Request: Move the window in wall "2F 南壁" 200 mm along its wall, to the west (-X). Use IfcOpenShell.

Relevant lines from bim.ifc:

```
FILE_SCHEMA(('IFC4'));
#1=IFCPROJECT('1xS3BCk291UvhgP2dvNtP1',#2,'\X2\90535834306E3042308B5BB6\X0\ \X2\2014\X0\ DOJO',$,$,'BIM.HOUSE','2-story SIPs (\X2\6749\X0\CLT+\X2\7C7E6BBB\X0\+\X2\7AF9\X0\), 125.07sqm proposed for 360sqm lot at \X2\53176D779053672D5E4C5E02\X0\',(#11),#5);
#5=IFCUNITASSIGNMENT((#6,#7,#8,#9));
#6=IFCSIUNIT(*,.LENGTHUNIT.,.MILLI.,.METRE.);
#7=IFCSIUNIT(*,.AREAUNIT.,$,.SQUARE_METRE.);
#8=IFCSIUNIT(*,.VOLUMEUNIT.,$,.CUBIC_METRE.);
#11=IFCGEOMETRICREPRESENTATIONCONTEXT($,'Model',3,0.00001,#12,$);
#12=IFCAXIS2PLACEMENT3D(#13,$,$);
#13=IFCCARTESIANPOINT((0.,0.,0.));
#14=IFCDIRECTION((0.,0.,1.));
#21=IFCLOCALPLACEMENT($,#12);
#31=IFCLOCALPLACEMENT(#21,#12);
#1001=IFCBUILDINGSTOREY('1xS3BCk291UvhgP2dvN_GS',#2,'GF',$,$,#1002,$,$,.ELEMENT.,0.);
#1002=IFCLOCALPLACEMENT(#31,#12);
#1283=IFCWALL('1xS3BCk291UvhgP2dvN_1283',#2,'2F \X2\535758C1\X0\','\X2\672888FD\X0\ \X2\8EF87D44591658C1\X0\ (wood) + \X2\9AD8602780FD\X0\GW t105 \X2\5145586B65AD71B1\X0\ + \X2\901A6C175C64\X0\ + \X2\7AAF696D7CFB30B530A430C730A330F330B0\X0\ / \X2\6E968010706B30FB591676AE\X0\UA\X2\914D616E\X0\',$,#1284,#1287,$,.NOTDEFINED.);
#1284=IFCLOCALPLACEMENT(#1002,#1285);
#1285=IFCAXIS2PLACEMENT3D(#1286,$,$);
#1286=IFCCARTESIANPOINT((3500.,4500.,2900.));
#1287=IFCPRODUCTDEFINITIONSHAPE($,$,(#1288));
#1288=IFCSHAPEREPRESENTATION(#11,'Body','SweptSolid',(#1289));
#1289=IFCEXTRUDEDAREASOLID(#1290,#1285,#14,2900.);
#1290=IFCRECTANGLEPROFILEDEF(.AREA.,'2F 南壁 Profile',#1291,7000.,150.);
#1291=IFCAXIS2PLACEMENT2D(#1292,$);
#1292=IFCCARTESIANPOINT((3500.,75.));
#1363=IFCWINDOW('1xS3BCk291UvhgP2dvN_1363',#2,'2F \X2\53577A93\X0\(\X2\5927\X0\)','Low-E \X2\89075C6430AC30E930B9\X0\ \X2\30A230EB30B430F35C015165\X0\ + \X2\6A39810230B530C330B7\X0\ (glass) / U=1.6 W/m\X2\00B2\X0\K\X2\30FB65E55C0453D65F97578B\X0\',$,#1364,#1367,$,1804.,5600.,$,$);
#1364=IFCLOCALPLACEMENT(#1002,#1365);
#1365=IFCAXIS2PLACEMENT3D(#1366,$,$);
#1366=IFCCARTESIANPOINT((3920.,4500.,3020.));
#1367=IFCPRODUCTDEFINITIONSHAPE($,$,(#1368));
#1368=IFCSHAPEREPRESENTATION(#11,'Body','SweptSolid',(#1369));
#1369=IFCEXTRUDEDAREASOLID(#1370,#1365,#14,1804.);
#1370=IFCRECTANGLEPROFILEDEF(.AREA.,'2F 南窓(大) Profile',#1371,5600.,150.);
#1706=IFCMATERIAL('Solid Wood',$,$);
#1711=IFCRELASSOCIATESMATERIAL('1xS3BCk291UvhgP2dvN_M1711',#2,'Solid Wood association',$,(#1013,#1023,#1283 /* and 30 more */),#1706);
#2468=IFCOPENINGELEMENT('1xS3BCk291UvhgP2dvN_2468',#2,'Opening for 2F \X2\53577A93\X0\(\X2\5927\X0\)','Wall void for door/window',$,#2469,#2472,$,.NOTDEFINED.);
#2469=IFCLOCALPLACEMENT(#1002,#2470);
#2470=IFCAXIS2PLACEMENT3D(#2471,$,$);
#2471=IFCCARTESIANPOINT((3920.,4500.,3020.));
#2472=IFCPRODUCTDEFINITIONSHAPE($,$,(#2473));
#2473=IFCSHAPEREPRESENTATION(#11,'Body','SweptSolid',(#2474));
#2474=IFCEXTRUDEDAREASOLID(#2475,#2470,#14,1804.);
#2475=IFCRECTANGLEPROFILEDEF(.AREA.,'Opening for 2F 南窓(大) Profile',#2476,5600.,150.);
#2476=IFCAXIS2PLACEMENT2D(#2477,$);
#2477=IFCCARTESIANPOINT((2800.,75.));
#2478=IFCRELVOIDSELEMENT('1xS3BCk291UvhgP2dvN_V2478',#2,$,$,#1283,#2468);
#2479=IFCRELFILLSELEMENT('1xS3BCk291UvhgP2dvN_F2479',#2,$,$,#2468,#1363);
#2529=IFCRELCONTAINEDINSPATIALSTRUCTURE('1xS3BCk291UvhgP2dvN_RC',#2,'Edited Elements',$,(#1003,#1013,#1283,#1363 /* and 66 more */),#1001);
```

```python
import ifcopenshell
import ifcopenshell.api.geometry
import ifcopenshell.util.placement
import ifcopenshell.util.unit

model = ifcopenshell.open("bim.ifc")
unit_scale = ifcopenshell.util.unit.calculate_unit_scale(model)

window = model.by_id(1363)
opening = window.FillsVoids[0].RelatingOpeningElement
wall = opening.VoidsElements[0].RelatingBuildingElement

wall_matrix = ifcopenshell.util.placement.get_local_placement(wall.ObjectPlacement)
shift = wall_matrix[:3, 0] * -0.2 / unit_scale
before = ifcopenshell.util.placement.get_local_placement(window.ObjectPlacement)[:3, 3].copy()

# The window is not placed relative to its opening, so move both.
for product in (opening, window):
    matrix = ifcopenshell.util.placement.get_local_placement(product.ObjectPlacement)
    matrix[:3, 3] += shift
    ifcopenshell.api.geometry.edit_object_placement(model, product=product, matrix=matrix, is_si=False)

after = ifcopenshell.util.placement.get_local_placement(window.ObjectPlacement)[:3, 3]
print("window moved by", (after - before).round(3) + 0.0)

model.write("bim_edited.ifc")
```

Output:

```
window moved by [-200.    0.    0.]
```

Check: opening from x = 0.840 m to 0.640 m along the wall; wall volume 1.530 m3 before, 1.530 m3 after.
